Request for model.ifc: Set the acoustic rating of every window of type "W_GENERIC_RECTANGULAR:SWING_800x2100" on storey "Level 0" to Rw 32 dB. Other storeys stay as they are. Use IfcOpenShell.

First a look at what the model holds.

```python
import ifcopenshell
import ifcopenshell.util.element

model = ifcopenshell.open("model.ifc")
print(model.schema)
storey = next(s for s in model.by_type("IfcBuildingStorey") if s.Name == "Level 0")
windows = [e for e in ifcopenshell.util.element.get_decomposition(storey) if e.is_a("IfcWindow")]
seen = {}
for e in windows:
    element_type = ifcopenshell.util.element.get_type(e)
    key = (element_type.Name if element_type != e and element_type else None, ifcopenshell.util.element.get_pset(e, "Pset_WindowCommon", "AcousticRating"))
    seen[key] = seen.get(key, 0) + 1
for (name, value), count in sorted(seen.items(), key=str):
    print(count, "x", name, "|", value)
```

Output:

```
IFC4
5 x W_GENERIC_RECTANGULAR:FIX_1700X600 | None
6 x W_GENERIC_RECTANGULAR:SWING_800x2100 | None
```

```python
import ifcopenshell
import ifcopenshell.api.pset
import ifcopenshell.util.element

model = ifcopenshell.open("model.ifc")

storey = next(s for s in model.by_type("IfcBuildingStorey") if s.Name == "Level 0")
windows = [e for e in ifcopenshell.util.element.get_decomposition(storey) if e.is_a("IfcWindow")]

count = 0
for e in windows:
    element_type = ifcopenshell.util.element.get_type(e)
    if element_type in (None, e) or element_type.Name != "W_GENERIC_RECTANGULAR:SWING_800x2100":
        continue
    # add_pset returns the element's existing set when there is one.
    pset = ifcopenshell.api.pset.add_pset(model, product=e, name="Pset_WindowCommon")
    ifcopenshell.api.pset.edit_pset(model, pset=pset, properties={"AcousticRating": "Rw 32 dB"})
    count += 1

print(count, "windows updated")

model.write("model_rev.ifc")
```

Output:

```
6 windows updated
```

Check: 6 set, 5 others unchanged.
